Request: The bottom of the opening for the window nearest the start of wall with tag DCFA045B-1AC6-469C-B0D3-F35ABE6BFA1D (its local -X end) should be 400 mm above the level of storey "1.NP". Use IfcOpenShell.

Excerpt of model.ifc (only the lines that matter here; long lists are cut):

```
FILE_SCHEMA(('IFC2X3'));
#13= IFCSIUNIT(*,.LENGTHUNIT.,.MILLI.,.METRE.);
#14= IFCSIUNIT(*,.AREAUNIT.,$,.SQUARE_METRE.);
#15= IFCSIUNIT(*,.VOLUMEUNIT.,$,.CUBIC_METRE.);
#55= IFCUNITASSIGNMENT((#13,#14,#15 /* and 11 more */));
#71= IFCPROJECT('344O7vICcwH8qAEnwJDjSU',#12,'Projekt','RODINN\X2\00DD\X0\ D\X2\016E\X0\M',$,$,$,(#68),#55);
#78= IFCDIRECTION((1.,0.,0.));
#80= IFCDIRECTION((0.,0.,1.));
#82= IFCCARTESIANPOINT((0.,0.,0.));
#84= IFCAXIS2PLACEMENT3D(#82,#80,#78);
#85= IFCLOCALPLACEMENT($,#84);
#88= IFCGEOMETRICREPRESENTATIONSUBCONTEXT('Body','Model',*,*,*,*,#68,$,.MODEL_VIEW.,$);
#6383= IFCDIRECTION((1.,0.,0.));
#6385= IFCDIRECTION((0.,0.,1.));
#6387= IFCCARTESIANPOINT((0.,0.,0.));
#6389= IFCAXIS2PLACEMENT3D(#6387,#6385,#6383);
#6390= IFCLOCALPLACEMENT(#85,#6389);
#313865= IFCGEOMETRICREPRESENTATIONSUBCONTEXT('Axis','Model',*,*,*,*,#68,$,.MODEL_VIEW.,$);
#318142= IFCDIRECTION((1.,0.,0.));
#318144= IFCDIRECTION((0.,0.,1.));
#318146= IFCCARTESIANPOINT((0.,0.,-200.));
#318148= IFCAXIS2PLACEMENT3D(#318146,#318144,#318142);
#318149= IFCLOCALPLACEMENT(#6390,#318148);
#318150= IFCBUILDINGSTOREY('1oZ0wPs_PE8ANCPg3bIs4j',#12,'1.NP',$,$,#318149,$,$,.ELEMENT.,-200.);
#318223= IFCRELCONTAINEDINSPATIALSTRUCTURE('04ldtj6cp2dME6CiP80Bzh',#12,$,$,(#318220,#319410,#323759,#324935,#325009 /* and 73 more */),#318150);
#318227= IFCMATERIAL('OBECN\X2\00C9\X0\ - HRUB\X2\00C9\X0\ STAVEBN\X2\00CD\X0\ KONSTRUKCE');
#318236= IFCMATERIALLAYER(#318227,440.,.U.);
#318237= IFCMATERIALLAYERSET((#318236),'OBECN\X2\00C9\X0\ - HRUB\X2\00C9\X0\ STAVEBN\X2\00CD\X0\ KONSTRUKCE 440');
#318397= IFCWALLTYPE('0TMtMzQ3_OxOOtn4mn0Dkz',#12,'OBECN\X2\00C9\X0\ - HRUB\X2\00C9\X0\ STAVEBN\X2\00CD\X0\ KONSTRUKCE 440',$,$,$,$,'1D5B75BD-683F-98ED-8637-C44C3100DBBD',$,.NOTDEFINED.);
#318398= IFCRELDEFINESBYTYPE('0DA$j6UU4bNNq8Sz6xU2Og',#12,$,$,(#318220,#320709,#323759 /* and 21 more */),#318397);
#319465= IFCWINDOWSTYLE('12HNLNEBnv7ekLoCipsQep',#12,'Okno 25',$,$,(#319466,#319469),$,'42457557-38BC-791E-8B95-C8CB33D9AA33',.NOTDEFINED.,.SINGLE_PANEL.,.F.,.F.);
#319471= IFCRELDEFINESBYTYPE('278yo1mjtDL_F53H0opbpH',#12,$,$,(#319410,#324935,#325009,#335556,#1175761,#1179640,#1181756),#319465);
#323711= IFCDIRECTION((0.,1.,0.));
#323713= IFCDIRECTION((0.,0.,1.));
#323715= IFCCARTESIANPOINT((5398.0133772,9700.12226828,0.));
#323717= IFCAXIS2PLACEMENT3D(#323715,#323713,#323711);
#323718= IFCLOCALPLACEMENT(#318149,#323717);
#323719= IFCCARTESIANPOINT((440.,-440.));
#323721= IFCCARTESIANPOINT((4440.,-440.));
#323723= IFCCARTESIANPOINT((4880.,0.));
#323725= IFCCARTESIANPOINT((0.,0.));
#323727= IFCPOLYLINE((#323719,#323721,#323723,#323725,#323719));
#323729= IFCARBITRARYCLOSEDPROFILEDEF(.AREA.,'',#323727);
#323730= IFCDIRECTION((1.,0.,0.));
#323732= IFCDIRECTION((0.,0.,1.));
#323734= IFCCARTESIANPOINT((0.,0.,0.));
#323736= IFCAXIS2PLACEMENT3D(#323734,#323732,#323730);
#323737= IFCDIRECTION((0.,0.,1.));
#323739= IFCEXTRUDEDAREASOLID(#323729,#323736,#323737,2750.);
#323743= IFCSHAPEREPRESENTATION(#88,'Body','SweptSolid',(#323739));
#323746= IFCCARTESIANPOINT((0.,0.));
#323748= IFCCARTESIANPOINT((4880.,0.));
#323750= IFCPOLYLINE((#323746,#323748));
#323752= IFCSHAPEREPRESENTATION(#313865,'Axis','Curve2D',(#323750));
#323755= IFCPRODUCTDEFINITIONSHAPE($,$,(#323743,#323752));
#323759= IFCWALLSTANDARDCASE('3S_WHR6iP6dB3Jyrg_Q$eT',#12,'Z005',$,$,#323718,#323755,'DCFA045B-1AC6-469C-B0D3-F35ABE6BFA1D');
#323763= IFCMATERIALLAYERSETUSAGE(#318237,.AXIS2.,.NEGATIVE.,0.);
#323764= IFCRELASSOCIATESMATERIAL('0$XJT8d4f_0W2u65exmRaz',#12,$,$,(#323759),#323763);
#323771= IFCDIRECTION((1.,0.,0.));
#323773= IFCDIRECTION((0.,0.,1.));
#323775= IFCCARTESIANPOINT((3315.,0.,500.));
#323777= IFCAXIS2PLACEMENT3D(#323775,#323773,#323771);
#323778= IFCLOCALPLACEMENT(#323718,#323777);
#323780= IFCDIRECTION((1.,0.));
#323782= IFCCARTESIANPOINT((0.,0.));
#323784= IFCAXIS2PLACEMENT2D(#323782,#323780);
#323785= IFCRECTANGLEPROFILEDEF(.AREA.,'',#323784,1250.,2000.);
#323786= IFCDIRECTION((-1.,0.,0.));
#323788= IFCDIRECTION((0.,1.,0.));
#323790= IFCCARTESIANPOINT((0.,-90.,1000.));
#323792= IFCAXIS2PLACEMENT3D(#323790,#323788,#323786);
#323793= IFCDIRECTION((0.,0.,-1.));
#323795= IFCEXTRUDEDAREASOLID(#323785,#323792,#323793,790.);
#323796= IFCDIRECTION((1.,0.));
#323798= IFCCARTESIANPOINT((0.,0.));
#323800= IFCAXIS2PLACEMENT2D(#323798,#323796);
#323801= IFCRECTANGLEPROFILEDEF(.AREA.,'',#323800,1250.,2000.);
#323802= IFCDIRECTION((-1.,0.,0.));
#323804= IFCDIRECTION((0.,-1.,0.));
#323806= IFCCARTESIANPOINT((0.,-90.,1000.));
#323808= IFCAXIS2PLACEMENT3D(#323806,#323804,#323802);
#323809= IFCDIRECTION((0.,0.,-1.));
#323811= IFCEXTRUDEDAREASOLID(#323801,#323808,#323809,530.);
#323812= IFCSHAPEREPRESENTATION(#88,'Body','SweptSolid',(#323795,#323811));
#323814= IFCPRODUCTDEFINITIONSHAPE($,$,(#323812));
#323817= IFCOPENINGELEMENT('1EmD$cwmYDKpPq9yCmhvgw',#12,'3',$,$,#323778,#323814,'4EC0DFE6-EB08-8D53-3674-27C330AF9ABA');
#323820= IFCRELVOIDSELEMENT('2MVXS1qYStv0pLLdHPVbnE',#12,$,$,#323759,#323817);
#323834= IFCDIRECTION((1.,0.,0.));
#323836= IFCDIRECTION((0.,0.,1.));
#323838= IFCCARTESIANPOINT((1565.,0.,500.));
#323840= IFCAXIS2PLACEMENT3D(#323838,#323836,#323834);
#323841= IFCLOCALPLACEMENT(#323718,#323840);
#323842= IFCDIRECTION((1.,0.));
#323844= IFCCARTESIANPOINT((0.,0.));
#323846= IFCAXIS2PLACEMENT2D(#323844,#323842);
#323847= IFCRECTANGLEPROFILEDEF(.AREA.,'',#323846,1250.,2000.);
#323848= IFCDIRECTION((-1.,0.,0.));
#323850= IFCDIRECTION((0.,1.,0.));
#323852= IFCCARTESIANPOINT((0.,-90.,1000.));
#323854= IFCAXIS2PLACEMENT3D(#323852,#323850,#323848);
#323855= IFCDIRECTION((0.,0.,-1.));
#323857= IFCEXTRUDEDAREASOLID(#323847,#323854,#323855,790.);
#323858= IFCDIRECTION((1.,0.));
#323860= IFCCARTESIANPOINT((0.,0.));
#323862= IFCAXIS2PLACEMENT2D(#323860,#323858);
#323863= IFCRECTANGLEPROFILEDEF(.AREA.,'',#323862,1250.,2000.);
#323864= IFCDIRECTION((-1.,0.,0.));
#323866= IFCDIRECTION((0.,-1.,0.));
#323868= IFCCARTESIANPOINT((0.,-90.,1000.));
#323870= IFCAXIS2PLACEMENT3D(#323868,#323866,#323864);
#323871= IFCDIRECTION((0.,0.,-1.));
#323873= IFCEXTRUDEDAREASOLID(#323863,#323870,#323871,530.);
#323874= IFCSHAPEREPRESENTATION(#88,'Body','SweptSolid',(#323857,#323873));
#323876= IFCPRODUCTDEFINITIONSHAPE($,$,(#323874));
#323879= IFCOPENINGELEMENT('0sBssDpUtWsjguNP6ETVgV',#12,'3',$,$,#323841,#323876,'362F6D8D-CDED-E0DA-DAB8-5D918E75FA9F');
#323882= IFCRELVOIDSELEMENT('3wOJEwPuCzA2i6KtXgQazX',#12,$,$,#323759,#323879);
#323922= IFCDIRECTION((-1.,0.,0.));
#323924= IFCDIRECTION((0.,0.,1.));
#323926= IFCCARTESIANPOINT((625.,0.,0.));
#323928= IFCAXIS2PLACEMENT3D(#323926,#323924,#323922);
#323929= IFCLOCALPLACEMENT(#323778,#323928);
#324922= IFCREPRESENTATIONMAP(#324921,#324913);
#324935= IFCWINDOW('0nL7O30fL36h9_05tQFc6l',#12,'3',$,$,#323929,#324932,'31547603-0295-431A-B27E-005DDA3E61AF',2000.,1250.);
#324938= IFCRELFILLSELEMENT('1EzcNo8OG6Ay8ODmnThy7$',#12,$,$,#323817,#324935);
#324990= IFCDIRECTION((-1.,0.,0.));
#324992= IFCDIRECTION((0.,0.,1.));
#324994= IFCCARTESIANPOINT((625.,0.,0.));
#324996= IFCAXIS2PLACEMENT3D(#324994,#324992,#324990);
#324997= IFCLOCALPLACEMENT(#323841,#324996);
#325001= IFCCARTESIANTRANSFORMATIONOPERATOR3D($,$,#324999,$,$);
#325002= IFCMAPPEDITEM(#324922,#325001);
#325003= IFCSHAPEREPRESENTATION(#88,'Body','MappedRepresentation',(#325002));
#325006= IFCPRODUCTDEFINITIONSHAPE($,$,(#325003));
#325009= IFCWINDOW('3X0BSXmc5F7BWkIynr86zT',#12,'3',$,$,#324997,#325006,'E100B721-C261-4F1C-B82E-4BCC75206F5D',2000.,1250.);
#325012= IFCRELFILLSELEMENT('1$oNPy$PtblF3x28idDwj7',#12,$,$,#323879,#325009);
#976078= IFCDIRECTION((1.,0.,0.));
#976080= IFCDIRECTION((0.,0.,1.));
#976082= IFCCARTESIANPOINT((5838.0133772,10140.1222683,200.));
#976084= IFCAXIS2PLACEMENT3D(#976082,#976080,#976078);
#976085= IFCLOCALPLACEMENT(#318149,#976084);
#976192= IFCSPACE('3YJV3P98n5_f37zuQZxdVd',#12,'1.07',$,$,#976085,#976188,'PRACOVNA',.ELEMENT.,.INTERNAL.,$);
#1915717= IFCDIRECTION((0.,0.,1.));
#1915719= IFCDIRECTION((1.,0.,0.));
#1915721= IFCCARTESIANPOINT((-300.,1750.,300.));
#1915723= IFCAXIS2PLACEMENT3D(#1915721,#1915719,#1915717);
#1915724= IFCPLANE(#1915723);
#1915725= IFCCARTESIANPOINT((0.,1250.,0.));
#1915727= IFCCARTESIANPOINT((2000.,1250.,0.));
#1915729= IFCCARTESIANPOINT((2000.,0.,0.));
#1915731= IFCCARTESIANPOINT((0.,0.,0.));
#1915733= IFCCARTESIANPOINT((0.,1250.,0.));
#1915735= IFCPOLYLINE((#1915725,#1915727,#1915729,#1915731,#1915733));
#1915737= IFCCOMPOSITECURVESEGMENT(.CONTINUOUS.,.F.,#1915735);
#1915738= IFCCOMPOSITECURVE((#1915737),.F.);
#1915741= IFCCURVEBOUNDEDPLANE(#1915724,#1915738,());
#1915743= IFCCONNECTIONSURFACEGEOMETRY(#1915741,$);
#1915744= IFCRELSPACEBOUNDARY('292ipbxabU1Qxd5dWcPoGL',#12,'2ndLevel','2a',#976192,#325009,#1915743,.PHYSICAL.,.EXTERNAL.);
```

```python
import numpy as np
import ifcopenshell
import ifcopenshell.api.geometry
import ifcopenshell.geom
import ifcopenshell.util.element
import ifcopenshell.util.placement
import ifcopenshell.util.shape
import ifcopenshell.util.unit

model = ifcopenshell.open("model.ifc")
unit_scale = ifcopenshell.util.unit.calculate_unit_scale(model)

window = model.by_id(325009)
opening = window.FillsVoids[0].RelatingOpeningElement
storey = ifcopenshell.util.element.get_container(window, ifc_class="IfcBuildingStorey")
level = ifcopenshell.util.placement.get_local_placement(storey.ObjectPlacement)[2, 3]

# The opening's origin need not be at the sill, so measure its lowest point.
shape = ifcopenshell.geom.create_shape(ifcopenshell.geom.settings(), opening)
bottom = ifcopenshell.util.shape.get_shape_bottom_elevation(shape, shape.geometry) / unit_scale
dz = level + 0.4 / unit_scale - bottom

shift = np.array([0.0, 0.0, dz])
# The window is placed relative to its opening, so it follows when the opening moves.
matrix = ifcopenshell.util.placement.get_local_placement(opening.ObjectPlacement)
matrix[:3, 3] += shift
ifcopenshell.api.geometry.edit_object_placement(
    model, product=opening, matrix=matrix, is_si=False, should_transform_children=True
)

# Space boundary surfaces are stored in each space's coordinates; move them too.
for rel in window.ProvidesBoundaries:
    if not rel.ConnectionGeometry:
        continue
    surface = rel.ConnectionGeometry.SurfaceOnRelatingElement.BasisSurface
    space_matrix = ifcopenshell.util.placement.get_local_placement(rel.RelatingSpace.ObjectPlacement)
    point = np.array(surface.Position.Location.Coordinates) + space_matrix[:3, :3].T @ shift
    surface.Position = model.createIfcAxis2Placement3D(
        model.createIfcCartesianPoint(point.tolist()), surface.Position.Axis, surface.Position.RefDirection
    )

print(f"moved by {dz * unit_scale:+.3f} m")

model.write("model_rev.ifc")
```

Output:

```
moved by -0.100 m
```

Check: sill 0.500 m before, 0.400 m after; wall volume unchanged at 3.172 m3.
